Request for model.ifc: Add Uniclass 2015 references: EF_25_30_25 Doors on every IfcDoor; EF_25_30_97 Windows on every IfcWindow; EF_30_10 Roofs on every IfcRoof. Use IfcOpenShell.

First a look at what the model holds.

```python
import ifcopenshell

model = ifcopenshell.open("model.ifc")
print(model.schema)
print("classifications:", [c.Name for c in model.by_type("IfcClassification")])
for ifc_class in ("IfcDoor", "IfcRoof", "IfcStair", "IfcWall", "IfcWindow"):
    print(ifc_class, len(model.by_type(ifc_class)))
```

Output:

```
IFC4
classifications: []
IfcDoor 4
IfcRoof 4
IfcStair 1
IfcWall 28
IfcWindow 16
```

```python
import ifcopenshell
import ifcopenshell.api.classification

model = ifcopenshell.open("model.ifc")

system = ifcopenshell.api.classification.add_classification(model, classification="Uniclass 2015")

codes = {
    "IfcDoor": ("EF_25_30_25", "Doors"),
    "IfcWindow": ("EF_25_30_97", "Windows"),
    "IfcRoof": ("EF_30_10", "Roofs"),
}
for ifc_class, (code, name) in codes.items():
    products = model.by_type(ifc_class)
    ifcopenshell.api.classification.add_reference(
        model, products=products, classification=system, identification=code, name=name
    )
    print(code, len(products))

model.write("model_v2.ifc")
```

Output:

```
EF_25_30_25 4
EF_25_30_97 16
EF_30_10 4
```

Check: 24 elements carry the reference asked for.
